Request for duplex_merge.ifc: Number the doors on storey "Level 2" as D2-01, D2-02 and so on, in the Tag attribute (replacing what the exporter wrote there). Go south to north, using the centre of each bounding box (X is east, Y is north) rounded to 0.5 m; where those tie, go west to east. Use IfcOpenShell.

First a look at what the model holds.

```python
import ifcopenshell
import ifcopenshell.util.element
import ifcopenshell.util.placement

model = ifcopenshell.open("duplex_merge.ifc")
print(model.schema)
storey = next(s for s in model.by_type("IfcBuildingStorey") if s.Name == "Level 2")
doors = [e for e in ifcopenshell.util.element.get_decomposition(storey) if e.is_a("IfcDoor")]
for e in sorted(doors, key=lambda e: e.id()):
    origin = ifcopenshell.util.placement.get_local_placement(e.ObjectPlacement)[:3, 3]
    print(e.id(), e.Tag, e.Name, origin.round(2) + 0.0, sep=" | ")
```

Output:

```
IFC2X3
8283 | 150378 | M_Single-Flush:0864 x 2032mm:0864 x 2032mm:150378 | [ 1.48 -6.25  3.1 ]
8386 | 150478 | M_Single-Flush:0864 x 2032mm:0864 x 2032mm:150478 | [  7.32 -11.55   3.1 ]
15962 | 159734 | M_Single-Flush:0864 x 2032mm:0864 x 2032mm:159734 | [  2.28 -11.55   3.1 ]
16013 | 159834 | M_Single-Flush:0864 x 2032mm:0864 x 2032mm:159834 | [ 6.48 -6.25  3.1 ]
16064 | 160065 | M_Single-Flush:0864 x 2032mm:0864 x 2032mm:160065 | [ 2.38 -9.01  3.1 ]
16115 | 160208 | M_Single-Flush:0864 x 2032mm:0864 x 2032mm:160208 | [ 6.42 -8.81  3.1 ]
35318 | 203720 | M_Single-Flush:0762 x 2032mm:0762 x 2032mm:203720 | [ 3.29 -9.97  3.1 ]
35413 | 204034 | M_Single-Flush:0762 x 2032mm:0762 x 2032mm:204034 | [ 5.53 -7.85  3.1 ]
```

```python
import ifcopenshell
import ifcopenshell.geom
import ifcopenshell.util.element
import ifcopenshell.util.shape

model = ifcopenshell.open("duplex_merge.ifc")
settings = ifcopenshell.geom.settings()
settings.set("use-world-coords", True)


def centre(element):
    shape = ifcopenshell.geom.create_shape(settings, element)
    return ifcopenshell.util.shape.get_bbox_centroid(shape.geometry)


storey = next(s for s in model.by_type("IfcBuildingStorey") if s.Name == "Level 2")
doors = [e for e in ifcopenshell.util.element.get_decomposition(storey) if e.is_a("IfcDoor")]

# Insertion points can sit at a corner or the storey origin, so sort by the geometry (in metres).
centres = {e: centre(e) for e in doors}
doors.sort(key=lambda e: (round(centres[e][1] / 0.5), centres[e][0]))

for i, e in enumerate(doors, start=1):
    number = f"D2-{i:02d}"
    e.Tag = number
    print(e.id(), number)

model.write("duplex_merge_edited.ifc")
```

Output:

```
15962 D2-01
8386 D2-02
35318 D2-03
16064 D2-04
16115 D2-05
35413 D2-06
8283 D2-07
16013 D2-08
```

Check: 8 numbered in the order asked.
